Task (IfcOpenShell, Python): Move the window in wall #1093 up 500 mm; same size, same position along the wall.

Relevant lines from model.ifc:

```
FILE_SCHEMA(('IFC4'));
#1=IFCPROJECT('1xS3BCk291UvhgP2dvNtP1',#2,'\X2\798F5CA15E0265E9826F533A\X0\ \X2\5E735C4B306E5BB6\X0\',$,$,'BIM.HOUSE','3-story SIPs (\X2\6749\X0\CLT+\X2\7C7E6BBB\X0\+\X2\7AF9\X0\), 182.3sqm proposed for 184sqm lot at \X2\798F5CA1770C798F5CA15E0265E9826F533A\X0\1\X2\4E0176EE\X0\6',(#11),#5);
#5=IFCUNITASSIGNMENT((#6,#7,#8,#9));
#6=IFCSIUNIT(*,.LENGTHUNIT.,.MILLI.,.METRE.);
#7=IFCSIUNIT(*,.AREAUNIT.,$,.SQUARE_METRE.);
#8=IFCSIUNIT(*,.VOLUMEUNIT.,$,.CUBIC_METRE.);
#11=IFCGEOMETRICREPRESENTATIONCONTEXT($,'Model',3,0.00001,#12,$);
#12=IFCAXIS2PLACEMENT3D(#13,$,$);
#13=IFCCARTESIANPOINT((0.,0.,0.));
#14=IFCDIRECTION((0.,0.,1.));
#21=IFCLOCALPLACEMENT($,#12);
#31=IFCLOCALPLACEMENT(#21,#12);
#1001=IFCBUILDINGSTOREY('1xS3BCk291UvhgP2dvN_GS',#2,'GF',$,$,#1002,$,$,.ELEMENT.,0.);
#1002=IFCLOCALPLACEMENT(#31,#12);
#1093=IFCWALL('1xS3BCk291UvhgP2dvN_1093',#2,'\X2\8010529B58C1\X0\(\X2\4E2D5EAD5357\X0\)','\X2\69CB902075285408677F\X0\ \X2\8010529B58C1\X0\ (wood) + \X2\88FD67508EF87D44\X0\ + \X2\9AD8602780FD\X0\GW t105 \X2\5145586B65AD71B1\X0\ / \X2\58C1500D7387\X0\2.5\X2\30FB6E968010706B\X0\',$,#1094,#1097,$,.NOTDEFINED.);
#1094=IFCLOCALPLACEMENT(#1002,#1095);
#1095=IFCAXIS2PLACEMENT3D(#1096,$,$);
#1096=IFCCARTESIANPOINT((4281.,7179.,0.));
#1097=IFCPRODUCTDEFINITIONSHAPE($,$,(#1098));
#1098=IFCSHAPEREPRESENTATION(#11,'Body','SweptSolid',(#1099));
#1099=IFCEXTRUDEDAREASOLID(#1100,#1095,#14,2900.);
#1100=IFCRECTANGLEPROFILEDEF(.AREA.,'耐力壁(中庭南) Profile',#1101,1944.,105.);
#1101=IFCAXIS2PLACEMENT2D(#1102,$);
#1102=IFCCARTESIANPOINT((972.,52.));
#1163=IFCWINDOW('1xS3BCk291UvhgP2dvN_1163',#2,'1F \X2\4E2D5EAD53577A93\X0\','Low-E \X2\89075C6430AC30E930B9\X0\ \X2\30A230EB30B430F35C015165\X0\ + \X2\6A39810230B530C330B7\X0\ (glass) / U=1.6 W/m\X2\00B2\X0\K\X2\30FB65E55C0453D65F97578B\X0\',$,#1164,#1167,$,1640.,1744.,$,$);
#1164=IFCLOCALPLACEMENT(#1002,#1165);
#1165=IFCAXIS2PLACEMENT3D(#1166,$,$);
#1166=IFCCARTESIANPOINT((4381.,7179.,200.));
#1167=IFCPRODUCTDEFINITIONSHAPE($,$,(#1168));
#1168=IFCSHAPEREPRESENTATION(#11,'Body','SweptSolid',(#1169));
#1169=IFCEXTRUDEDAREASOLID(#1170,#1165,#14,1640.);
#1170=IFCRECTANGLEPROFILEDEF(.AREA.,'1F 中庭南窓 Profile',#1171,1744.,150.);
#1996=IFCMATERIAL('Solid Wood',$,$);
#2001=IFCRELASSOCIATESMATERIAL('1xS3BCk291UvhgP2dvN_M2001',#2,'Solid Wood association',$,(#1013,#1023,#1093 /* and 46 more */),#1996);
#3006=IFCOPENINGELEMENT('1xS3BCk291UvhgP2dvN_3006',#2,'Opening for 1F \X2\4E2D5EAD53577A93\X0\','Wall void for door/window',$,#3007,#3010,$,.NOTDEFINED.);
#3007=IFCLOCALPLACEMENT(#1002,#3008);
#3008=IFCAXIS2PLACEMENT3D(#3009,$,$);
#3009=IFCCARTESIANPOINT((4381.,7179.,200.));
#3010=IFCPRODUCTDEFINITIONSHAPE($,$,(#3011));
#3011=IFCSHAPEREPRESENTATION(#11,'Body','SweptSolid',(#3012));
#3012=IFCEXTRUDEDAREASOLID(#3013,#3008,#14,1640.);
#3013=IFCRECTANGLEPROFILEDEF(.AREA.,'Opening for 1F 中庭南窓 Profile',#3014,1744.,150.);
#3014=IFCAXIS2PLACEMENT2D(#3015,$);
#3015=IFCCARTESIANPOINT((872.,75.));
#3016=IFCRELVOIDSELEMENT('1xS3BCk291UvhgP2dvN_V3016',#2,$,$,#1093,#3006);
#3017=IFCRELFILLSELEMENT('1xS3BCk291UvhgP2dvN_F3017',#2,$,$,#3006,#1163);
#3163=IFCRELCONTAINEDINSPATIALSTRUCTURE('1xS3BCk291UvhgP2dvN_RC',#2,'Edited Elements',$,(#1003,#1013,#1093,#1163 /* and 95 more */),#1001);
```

```python
import numpy as np
import ifcopenshell
import ifcopenshell.api.geometry
import ifcopenshell.util.placement
import ifcopenshell.util.unit

model = ifcopenshell.open("model.ifc")
unit_scale = ifcopenshell.util.unit.calculate_unit_scale(model)

window = model.by_guid("1xS3BCk291UvhgP2dvN_1163")
opening = window.FillsVoids[0].RelatingOpeningElement
dz = 0.5 / unit_scale

shift = np.array([0.0, 0.0, dz])
# The window is not placed relative to its opening, so move both.
for product in (opening, window):
    matrix = ifcopenshell.util.placement.get_local_placement(product.ObjectPlacement)
    matrix[:3, 3] += shift
    ifcopenshell.api.geometry.edit_object_placement(model, product=product, matrix=matrix, is_si=False)

print(f"moved by {dz * unit_scale:+.3f} m")

model.write("model_v2.ifc")
```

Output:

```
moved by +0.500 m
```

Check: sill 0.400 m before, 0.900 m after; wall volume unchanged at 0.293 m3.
